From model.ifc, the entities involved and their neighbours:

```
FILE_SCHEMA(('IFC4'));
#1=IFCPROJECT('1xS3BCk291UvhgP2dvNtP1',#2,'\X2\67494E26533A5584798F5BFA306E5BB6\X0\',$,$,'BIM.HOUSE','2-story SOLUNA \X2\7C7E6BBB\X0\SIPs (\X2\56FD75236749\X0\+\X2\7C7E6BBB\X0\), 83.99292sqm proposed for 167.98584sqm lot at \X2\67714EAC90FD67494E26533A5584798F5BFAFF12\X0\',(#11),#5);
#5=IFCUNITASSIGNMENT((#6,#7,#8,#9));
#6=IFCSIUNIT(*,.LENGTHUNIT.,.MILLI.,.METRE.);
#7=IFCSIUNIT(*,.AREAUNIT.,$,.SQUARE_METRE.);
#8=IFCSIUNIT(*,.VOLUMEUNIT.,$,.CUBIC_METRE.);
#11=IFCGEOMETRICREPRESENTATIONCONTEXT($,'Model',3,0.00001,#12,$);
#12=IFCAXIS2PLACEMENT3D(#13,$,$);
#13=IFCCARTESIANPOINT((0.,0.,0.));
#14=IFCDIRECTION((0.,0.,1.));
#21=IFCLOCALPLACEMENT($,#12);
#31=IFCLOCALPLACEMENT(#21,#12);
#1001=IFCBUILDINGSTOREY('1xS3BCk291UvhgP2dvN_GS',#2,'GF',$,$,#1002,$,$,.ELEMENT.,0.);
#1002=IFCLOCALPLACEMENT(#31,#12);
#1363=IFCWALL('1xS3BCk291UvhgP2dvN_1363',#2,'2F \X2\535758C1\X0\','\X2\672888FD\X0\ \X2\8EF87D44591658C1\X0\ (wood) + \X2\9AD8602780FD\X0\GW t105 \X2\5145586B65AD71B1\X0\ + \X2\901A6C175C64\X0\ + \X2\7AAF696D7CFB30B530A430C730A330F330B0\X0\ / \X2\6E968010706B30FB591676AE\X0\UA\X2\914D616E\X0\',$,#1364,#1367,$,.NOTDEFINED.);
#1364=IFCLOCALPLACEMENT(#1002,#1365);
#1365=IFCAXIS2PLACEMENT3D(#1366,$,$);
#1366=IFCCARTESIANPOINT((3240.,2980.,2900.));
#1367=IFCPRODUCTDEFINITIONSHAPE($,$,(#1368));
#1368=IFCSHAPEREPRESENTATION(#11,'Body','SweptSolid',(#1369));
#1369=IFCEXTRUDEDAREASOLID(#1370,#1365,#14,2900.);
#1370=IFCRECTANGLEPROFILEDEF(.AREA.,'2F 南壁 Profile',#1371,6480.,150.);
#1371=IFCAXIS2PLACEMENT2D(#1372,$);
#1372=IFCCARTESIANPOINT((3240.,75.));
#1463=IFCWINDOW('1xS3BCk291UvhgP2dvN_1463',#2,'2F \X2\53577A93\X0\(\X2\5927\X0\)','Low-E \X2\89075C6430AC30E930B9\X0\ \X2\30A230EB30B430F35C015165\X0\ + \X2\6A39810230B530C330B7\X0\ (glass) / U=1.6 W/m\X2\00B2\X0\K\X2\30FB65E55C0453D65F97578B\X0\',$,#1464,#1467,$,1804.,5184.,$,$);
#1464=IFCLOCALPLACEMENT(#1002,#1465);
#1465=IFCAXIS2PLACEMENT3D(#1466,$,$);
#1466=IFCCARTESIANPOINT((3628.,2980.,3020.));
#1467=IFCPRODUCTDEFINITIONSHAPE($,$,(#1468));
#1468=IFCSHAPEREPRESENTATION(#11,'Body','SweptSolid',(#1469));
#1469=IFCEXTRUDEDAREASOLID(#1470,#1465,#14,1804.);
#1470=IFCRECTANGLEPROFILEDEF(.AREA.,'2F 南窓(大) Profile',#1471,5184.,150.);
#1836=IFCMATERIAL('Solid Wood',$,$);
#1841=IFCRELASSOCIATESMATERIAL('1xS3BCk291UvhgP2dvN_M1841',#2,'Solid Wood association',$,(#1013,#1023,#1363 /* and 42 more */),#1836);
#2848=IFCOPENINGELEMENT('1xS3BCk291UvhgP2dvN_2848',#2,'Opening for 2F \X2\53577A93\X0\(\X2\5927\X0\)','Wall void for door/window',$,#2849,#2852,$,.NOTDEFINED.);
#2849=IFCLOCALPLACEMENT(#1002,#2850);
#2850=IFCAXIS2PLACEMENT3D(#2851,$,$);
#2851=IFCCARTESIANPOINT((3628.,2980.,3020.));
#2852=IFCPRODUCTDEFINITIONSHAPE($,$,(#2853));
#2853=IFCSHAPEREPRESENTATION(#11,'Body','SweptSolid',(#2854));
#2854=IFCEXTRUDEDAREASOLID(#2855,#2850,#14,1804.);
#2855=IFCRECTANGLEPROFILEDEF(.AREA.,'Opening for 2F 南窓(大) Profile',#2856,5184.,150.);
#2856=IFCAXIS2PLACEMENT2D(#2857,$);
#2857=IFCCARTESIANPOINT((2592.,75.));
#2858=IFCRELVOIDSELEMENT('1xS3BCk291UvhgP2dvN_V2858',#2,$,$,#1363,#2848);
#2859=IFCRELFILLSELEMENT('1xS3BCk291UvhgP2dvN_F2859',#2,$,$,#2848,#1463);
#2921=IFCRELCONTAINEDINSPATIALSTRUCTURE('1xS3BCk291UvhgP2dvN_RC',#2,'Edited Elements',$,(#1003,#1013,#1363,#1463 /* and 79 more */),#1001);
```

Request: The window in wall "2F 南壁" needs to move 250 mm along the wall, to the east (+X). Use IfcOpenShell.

```python
import ifcopenshell
import ifcopenshell.api.geometry
import ifcopenshell.util.placement
import ifcopenshell.util.unit

model = ifcopenshell.open("model.ifc")
unit_scale = ifcopenshell.util.unit.calculate_unit_scale(model)

window = model.by_guid("1xS3BCk291UvhgP2dvN_1463")
opening = window.FillsVoids[0].RelatingOpeningElement
wall = opening.VoidsElements[0].RelatingBuildingElement

wall_matrix = ifcopenshell.util.placement.get_local_placement(wall.ObjectPlacement)
shift = wall_matrix[:3, 0] * 0.25 / unit_scale
before = ifcopenshell.util.placement.get_local_placement(window.ObjectPlacement)[:3, 3].copy()

# The window is not placed relative to its opening, so move both.
for product in (opening, window):
    matrix = ifcopenshell.util.placement.get_local_placement(product.ObjectPlacement)
    matrix[:3, 3] += shift
    ifcopenshell.api.geometry.edit_object_placement(model, product=product, matrix=matrix, is_si=False)

after = ifcopenshell.util.placement.get_local_placement(window.ObjectPlacement)[:3, 3]
print("window moved by", (after - before).round(3) + 0.0)

model.write("model_edited.ifc")
```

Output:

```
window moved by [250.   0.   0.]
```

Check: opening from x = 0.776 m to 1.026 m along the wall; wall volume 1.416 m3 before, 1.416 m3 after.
